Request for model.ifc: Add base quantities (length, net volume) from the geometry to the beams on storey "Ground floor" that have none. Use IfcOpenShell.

First a look at what the model holds.

```python
import ifcopenshell
import ifcopenshell.util.element
import ifcopenshell.util.unit

model = ifcopenshell.open("model.ifc")
print(model.schema)
for unit_type in ("LENGTHUNIT", "AREAUNIT", "VOLUMEUNIT"):
    print(unit_type, ifcopenshell.util.unit.calculate_unit_scale(model, unit_type))
storey = next(s for s in model.by_type("IfcBuildingStorey") if s.Name == "Ground floor")
beams = [e for e in ifcopenshell.util.element.get_decomposition(storey) if e.is_a("IfcBeam")]
for e in sorted(beams, key=lambda e: e.id()):
    print(e.id(), e.is_a(), e.Name, list(ifcopenshell.util.element.get_psets(e, qtos_only=True)), sep=" | ")
```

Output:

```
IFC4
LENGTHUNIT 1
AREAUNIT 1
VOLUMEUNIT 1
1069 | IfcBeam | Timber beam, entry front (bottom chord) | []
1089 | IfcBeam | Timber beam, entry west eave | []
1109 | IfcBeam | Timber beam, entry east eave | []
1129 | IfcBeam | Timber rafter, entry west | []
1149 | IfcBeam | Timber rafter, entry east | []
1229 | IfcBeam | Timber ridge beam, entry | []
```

```python
import ifcopenshell
import ifcopenshell.api.pset
import ifcopenshell.geom
import ifcopenshell.util.element
import ifcopenshell.util.shape
import ifcopenshell.util.unit

model = ifcopenshell.open("model.ifc")
unit_scale = ifcopenshell.util.unit.calculate_unit_scale(model)
volume_scale = ifcopenshell.util.unit.calculate_unit_scale(model, "VOLUMEUNIT")
settings = ifcopenshell.geom.settings()

storey = next(s for s in model.by_type("IfcBuildingStorey") if s.Name == "Ground floor")
beams = [e for e in ifcopenshell.util.element.get_decomposition(storey) if e.is_a("IfcBeam")]

for e in sorted(beams, key=lambda e: e.id()):
    if ifcopenshell.util.element.get_psets(e, qtos_only=True, should_inherit=False):
        continue
    # Geometry comes back in metres, in the element's own axes.
    shape = ifcopenshell.geom.create_shape(settings, e)
    values = {
        "Length": ifcopenshell.util.shape.get_max_xyz(shape.geometry) / unit_scale,
        "NetVolume": ifcopenshell.util.shape.get_volume(shape.geometry) / volume_scale,
    }
    qto = ifcopenshell.api.pset.add_qto(model, product=e, name="Qto_BeamBaseQuantities")
    ifcopenshell.api.pset.edit_qto(model, qto=qto, properties=values)
    print(e.id(), {k: round(v, 3) for k, v in values.items()})

model.write("model_edited.ifc")
```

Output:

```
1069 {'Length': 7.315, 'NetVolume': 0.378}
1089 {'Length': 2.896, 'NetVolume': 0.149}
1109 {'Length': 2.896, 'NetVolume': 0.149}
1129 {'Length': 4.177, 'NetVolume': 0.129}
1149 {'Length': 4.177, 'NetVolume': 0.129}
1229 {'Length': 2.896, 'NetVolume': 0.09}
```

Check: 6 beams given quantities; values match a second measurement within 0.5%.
